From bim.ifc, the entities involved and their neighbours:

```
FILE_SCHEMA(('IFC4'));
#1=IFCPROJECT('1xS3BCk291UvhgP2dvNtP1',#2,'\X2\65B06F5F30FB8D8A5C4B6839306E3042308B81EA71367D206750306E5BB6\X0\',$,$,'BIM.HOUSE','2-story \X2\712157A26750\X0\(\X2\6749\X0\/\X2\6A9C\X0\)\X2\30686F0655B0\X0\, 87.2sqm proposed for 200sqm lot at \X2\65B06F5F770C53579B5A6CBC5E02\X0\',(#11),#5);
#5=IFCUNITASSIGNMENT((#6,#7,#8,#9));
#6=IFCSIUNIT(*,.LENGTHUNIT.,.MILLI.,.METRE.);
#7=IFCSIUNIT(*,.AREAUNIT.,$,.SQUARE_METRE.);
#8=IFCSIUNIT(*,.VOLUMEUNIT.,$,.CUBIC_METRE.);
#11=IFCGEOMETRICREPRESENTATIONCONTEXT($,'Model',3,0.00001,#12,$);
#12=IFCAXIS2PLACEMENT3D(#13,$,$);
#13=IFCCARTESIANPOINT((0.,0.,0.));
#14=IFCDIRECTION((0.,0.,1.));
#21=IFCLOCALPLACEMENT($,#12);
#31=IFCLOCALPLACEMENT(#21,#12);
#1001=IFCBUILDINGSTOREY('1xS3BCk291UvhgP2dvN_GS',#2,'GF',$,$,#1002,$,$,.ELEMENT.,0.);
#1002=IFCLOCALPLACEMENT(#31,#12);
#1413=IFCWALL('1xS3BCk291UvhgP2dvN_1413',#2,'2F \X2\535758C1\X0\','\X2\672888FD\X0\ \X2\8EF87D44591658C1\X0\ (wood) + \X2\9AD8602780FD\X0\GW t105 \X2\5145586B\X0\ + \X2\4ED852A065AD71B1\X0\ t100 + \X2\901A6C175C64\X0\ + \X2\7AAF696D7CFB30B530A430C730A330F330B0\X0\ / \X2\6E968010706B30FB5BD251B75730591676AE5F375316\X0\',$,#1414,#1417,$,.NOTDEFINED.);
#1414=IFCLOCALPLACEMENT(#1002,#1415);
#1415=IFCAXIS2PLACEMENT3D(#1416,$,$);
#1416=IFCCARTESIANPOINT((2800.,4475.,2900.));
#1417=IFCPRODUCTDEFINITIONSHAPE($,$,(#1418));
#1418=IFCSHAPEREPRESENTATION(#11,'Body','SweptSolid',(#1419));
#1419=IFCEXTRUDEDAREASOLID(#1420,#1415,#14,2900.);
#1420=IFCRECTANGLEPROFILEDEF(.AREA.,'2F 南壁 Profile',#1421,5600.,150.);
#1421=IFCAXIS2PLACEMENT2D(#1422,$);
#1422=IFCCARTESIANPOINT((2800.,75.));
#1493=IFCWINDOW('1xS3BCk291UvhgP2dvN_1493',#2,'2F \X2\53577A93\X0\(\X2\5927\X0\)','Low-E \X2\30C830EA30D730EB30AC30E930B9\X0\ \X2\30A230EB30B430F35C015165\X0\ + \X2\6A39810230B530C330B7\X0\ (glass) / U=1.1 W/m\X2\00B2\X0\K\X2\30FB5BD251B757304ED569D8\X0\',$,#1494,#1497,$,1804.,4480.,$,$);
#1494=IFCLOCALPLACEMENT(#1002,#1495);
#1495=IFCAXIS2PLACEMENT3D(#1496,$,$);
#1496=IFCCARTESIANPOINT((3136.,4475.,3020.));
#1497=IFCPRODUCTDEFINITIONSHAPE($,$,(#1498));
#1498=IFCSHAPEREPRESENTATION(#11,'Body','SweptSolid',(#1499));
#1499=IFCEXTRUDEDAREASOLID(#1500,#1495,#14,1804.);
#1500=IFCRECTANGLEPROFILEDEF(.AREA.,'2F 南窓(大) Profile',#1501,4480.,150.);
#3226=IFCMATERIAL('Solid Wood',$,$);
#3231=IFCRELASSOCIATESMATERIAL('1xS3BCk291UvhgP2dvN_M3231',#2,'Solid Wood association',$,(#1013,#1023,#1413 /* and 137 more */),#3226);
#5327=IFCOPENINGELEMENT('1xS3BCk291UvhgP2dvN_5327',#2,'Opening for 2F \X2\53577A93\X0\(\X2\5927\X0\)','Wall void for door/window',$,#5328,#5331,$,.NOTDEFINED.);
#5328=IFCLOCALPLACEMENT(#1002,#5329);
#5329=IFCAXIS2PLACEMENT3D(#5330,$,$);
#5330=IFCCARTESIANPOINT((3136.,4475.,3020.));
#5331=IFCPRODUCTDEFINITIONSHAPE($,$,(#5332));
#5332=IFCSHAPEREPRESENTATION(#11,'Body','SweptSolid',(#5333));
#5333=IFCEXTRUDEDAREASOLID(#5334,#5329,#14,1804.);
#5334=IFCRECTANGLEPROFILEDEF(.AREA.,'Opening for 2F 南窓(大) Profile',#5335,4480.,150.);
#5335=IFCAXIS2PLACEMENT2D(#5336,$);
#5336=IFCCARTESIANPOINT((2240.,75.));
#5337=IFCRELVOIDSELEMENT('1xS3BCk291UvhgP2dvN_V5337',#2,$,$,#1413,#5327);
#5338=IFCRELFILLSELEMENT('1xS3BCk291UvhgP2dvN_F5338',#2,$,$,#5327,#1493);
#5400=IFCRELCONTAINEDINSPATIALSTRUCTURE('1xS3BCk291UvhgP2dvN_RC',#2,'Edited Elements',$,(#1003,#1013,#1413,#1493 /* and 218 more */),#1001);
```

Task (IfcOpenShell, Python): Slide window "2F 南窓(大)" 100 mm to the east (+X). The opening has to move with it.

```python
import ifcopenshell
import ifcopenshell.api.geometry
import ifcopenshell.util.placement

model = ifcopenshell.open("bim.ifc")

window = model.by_id(1493)
opening = window.FillsVoids[0].RelatingOpeningElement
wall = opening.VoidsElements[0].RelatingBuildingElement

wall_matrix = ifcopenshell.util.placement.get_local_placement(wall.ObjectPlacement)
shift = wall_matrix[:3, 0] * 100.0
before = ifcopenshell.util.placement.get_local_placement(window.ObjectPlacement)[:3, 3].copy()

# The window is not placed relative to its opening, so move both.
for product in (opening, window):
    matrix = ifcopenshell.util.placement.get_local_placement(product.ObjectPlacement)
    matrix[:3, 3] += shift
    ifcopenshell.api.geometry.edit_object_placement(model, product=product, matrix=matrix, is_si=False)

after = ifcopenshell.util.placement.get_local_placement(window.ObjectPlacement)[:3, 3]
print("window moved by", (after - before).round(3) + 0.0)

model.write("bim_edited.ifc")
```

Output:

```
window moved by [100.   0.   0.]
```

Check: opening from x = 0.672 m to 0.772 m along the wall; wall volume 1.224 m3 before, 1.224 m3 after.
